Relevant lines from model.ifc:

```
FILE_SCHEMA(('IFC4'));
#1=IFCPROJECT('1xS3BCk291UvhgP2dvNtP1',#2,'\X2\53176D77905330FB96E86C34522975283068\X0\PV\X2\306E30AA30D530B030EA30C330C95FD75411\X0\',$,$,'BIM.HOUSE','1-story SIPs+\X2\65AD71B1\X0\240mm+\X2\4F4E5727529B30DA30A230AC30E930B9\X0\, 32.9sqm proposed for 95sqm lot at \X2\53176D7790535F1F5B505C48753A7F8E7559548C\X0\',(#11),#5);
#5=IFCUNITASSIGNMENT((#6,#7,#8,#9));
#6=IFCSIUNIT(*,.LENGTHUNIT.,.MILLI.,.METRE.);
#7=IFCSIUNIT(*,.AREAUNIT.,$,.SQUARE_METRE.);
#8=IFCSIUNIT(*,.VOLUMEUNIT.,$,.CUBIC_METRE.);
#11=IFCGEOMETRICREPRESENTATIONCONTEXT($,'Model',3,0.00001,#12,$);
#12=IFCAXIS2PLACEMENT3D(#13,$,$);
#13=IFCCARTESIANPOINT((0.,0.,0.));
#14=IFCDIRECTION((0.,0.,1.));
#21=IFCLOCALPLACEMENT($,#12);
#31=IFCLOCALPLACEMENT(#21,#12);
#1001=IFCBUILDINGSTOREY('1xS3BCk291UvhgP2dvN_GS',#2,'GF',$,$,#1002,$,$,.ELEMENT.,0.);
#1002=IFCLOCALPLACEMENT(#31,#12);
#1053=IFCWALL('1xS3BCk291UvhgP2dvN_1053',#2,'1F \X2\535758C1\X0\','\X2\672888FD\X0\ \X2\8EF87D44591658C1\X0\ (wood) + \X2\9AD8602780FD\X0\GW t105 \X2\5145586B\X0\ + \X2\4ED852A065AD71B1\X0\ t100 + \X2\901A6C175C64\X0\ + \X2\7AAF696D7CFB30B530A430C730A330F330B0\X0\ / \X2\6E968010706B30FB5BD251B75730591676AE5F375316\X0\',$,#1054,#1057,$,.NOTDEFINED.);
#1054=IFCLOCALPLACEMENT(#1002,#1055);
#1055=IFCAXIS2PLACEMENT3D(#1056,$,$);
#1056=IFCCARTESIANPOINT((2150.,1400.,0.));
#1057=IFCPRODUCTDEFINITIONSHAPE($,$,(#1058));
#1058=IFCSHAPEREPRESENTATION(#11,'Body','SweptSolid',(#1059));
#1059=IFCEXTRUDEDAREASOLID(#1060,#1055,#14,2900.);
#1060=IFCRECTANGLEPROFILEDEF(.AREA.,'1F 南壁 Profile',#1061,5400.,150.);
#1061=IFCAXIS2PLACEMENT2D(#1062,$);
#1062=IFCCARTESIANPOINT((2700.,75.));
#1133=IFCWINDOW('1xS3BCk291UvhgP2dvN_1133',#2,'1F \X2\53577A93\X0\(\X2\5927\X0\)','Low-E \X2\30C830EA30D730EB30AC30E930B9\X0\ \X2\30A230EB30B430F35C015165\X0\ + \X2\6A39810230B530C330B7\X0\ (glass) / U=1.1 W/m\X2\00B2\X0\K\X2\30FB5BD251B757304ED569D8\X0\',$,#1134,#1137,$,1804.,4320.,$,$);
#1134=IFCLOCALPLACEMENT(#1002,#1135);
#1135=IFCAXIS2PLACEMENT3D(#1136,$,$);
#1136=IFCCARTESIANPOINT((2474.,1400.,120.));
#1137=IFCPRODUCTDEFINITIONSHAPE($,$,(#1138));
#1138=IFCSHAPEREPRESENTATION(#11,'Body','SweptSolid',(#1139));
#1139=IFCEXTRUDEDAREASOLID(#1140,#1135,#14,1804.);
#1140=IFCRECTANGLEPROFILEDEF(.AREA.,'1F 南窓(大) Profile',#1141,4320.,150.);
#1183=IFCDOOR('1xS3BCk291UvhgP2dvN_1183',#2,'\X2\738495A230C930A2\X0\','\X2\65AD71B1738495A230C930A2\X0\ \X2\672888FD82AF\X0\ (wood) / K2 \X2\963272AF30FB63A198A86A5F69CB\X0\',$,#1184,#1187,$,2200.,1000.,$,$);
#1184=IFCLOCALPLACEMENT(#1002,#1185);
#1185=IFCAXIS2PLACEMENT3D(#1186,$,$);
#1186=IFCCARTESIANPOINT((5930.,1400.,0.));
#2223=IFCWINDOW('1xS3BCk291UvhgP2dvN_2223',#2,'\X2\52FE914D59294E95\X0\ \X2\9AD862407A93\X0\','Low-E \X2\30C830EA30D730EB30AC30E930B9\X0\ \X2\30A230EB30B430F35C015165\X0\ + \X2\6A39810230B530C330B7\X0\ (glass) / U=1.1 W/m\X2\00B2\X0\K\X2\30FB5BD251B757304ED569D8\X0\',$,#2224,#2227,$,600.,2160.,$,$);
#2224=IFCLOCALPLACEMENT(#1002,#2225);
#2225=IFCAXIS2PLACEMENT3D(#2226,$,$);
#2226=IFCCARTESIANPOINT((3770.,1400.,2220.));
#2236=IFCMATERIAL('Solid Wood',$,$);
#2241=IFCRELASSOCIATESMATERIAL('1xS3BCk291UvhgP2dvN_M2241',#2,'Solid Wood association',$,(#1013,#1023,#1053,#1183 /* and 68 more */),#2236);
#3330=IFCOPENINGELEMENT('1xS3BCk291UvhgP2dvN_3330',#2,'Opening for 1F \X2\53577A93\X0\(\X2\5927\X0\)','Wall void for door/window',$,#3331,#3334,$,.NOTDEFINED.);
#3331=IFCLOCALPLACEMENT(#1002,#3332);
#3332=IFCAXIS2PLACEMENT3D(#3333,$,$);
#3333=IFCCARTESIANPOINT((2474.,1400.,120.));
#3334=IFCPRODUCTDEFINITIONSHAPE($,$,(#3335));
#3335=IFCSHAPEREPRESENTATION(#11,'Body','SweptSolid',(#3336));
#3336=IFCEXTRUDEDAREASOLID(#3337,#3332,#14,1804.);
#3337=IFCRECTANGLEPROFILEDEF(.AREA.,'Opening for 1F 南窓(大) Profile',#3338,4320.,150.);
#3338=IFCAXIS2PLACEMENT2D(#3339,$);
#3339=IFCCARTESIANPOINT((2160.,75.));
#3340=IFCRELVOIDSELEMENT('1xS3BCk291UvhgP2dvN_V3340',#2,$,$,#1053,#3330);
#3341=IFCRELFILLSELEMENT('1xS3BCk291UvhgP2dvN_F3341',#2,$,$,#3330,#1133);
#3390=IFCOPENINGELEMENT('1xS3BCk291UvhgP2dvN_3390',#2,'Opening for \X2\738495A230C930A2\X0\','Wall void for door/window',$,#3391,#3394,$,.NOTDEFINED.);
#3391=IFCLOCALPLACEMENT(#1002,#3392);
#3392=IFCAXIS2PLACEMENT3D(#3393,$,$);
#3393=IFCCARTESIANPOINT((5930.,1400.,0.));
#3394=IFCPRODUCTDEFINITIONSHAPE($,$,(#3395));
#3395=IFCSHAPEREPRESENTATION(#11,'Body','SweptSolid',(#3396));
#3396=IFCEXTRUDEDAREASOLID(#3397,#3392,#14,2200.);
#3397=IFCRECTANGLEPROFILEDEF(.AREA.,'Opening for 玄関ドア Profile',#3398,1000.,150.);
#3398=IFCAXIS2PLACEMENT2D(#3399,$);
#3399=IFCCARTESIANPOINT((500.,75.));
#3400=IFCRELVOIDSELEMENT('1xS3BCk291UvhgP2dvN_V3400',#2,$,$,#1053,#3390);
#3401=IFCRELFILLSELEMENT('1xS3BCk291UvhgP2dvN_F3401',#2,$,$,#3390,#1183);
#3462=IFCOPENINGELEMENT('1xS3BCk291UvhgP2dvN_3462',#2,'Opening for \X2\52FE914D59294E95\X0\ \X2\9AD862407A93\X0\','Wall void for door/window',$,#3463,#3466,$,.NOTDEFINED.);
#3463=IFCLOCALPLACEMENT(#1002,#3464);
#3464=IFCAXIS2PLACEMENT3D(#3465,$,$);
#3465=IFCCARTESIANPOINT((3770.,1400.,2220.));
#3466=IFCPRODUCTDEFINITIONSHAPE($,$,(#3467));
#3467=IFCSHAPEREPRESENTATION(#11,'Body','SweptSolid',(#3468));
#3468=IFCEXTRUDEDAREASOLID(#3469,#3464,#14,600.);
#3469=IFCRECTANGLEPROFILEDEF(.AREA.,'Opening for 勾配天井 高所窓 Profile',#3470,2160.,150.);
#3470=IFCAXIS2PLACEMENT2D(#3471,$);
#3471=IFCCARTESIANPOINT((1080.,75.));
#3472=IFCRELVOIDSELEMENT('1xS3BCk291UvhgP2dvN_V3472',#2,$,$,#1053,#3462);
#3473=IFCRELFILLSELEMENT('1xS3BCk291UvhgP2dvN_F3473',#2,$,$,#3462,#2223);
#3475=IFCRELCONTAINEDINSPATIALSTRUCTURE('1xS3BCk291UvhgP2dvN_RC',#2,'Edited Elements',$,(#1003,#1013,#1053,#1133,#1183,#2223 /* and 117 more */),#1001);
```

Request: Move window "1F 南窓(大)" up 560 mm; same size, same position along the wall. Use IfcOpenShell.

```python
import numpy as np
import ifcopenshell
import ifcopenshell.api.geometry
import ifcopenshell.util.placement
import ifcopenshell.util.unit

model = ifcopenshell.open("model.ifc")
unit_scale = ifcopenshell.util.unit.calculate_unit_scale(model)

window = model.by_id(1133)
opening = window.FillsVoids[0].RelatingOpeningElement
dz = 0.56 / unit_scale

shift = np.array([0.0, 0.0, dz])
# The window is not placed relative to its opening, so move both.
for product in (opening, window):
    matrix = ifcopenshell.util.placement.get_local_placement(product.ObjectPlacement)
    matrix[:3, 3] += shift
    ifcopenshell.api.geometry.edit_object_placement(model, product=product, matrix=matrix, is_si=False)

print(f"moved by {dz * unit_scale:+.3f} m")

model.write("model-out.ifc")
```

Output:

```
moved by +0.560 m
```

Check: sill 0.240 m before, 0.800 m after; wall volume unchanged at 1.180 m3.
